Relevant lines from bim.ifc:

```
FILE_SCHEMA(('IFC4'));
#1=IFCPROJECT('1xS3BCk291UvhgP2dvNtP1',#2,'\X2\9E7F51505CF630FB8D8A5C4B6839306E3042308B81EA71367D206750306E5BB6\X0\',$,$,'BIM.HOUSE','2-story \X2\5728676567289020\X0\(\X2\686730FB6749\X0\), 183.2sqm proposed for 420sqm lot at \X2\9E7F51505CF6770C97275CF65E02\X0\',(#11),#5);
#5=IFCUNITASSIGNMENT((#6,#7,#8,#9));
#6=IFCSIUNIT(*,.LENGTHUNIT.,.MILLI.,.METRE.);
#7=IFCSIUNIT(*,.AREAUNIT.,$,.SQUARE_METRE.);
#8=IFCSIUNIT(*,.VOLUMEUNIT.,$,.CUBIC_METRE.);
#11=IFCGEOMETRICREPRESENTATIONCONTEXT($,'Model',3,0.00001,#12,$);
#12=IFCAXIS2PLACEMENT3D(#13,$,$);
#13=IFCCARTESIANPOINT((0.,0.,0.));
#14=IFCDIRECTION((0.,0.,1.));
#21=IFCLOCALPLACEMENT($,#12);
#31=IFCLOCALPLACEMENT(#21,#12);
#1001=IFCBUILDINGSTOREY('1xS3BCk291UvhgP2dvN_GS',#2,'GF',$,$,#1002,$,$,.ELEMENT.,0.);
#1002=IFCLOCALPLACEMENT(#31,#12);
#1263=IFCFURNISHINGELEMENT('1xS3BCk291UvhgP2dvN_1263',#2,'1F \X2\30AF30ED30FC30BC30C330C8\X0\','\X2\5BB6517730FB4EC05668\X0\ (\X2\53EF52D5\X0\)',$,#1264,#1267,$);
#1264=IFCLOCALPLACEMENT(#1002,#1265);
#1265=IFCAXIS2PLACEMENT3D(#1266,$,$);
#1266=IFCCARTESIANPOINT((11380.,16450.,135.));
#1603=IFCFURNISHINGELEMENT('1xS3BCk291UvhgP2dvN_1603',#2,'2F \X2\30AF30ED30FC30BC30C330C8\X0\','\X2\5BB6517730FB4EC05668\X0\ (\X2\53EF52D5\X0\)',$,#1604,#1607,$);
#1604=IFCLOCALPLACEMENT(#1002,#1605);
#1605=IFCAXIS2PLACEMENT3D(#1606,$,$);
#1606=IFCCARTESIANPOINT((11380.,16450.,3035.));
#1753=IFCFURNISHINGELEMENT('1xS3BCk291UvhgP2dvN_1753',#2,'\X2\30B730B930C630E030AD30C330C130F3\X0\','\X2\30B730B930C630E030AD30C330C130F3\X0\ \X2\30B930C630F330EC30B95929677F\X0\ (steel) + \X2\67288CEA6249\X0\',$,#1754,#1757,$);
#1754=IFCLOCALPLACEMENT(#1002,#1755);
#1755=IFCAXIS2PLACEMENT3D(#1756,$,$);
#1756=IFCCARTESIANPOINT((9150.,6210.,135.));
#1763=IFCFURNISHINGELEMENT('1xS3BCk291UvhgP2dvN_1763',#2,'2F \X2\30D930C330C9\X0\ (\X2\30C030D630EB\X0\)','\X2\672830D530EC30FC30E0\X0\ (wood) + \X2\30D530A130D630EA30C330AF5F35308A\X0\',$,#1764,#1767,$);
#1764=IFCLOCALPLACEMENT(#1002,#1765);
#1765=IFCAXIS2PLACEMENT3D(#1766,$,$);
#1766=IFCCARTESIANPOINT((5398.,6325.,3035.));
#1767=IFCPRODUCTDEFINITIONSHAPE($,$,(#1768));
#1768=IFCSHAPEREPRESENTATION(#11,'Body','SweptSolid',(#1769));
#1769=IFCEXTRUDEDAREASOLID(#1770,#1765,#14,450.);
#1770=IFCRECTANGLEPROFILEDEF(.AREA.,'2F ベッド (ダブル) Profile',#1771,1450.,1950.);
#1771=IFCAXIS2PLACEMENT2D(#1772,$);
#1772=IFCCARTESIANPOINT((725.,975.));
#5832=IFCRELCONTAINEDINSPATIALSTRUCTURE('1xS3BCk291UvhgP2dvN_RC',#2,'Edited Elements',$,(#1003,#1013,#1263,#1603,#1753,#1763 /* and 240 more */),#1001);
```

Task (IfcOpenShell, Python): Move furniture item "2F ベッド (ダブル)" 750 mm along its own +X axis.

```python
import ifcopenshell
import ifcopenshell.api.geometry
import ifcopenshell.util.placement

model = ifcopenshell.open("bim.ifc")

item = model.by_guid("1xS3BCk291UvhgP2dvN_1763")
matrix = ifcopenshell.util.placement.get_local_placement(item.ObjectPlacement)
matrix[:3, 3] += matrix[:3, 0] * 750.0
ifcopenshell.api.geometry.edit_object_placement(model, product=item, matrix=matrix, is_si=False)

print(ifcopenshell.util.placement.get_local_placement(item.ObjectPlacement).round(3) + 0.0)

model.write("bim_v2.ifc")
```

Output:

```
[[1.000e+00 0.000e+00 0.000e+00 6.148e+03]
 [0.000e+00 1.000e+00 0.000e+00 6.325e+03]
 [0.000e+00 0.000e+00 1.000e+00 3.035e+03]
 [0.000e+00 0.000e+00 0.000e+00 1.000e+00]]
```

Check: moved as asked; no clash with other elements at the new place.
